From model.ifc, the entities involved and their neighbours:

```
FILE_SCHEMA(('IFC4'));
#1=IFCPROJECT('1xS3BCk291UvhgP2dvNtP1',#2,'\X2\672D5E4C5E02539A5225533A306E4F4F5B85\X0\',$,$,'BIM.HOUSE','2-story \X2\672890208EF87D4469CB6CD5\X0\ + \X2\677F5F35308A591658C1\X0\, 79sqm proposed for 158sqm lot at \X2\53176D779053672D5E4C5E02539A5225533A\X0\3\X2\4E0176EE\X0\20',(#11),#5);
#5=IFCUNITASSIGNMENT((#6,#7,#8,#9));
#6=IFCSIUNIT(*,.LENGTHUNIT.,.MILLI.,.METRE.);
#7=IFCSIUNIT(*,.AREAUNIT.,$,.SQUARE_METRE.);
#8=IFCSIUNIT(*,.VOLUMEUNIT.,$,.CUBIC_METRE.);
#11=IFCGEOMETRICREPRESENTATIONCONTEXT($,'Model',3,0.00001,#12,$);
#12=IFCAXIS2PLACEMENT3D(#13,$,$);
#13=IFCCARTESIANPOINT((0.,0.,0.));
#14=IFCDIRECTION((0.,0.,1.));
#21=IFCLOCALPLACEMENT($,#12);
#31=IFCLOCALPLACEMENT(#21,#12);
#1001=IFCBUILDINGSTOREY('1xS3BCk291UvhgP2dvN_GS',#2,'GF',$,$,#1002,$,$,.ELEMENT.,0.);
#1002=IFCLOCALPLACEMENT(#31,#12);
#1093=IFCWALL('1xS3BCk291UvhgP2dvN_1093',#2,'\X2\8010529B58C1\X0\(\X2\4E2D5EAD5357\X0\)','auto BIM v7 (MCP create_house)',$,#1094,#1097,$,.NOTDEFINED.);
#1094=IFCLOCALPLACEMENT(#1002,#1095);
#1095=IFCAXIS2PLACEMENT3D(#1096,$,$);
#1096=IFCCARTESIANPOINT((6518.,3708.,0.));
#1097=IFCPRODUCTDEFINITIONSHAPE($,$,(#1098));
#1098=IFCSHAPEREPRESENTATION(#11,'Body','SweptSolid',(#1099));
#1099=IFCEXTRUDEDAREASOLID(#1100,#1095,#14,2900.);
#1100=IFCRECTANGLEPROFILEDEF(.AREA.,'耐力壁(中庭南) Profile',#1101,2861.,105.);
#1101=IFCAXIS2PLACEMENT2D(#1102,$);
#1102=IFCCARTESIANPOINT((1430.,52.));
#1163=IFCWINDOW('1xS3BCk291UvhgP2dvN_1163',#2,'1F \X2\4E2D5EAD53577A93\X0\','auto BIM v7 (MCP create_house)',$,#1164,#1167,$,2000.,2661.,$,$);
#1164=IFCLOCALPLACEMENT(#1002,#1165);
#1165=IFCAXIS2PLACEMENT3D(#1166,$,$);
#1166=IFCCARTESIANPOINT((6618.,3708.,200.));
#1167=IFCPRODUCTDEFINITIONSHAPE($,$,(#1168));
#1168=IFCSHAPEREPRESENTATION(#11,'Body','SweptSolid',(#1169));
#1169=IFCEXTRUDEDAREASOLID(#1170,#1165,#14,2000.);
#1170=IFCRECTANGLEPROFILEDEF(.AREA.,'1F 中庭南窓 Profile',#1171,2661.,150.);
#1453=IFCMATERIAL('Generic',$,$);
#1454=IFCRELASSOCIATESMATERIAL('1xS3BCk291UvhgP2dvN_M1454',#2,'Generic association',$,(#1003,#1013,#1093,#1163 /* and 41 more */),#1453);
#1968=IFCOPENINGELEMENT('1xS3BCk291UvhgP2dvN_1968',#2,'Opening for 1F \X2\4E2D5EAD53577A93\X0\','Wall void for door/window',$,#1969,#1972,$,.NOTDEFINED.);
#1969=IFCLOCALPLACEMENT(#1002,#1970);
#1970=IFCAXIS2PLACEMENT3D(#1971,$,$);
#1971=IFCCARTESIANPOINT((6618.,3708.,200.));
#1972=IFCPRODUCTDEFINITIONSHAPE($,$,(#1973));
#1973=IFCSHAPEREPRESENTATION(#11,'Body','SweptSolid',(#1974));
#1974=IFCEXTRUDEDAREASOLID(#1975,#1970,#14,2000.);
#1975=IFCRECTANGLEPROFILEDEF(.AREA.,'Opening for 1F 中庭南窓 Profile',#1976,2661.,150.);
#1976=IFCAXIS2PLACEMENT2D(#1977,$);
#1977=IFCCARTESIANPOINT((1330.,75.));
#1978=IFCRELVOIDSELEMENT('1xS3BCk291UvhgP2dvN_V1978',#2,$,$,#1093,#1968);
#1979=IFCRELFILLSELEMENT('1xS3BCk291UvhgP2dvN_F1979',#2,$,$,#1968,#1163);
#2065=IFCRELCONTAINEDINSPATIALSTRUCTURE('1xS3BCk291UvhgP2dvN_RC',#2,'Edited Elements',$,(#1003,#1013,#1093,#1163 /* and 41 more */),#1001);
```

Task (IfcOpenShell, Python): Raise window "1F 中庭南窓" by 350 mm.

```python
import numpy as np
import ifcopenshell
import ifcopenshell.api.geometry
import ifcopenshell.util.placement
import ifcopenshell.util.unit

model = ifcopenshell.open("model.ifc")
unit_scale = ifcopenshell.util.unit.calculate_unit_scale(model)

window = model.by_guid("1xS3BCk291UvhgP2dvN_1163")
opening = window.FillsVoids[0].RelatingOpeningElement
dz = 350.0

shift = np.array([0.0, 0.0, dz])
# The window is not placed relative to its opening, so move both.
for product in (opening, window):
    matrix = ifcopenshell.util.placement.get_local_placement(product.ObjectPlacement)
    matrix[:3, 3] += shift
    ifcopenshell.api.geometry.edit_object_placement(model, product=product, matrix=matrix, is_si=False)

print(f"moved by {dz * unit_scale:+.3f} m")

model.write("model-out.ifc")
```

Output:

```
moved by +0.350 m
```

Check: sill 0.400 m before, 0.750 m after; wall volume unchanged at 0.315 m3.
